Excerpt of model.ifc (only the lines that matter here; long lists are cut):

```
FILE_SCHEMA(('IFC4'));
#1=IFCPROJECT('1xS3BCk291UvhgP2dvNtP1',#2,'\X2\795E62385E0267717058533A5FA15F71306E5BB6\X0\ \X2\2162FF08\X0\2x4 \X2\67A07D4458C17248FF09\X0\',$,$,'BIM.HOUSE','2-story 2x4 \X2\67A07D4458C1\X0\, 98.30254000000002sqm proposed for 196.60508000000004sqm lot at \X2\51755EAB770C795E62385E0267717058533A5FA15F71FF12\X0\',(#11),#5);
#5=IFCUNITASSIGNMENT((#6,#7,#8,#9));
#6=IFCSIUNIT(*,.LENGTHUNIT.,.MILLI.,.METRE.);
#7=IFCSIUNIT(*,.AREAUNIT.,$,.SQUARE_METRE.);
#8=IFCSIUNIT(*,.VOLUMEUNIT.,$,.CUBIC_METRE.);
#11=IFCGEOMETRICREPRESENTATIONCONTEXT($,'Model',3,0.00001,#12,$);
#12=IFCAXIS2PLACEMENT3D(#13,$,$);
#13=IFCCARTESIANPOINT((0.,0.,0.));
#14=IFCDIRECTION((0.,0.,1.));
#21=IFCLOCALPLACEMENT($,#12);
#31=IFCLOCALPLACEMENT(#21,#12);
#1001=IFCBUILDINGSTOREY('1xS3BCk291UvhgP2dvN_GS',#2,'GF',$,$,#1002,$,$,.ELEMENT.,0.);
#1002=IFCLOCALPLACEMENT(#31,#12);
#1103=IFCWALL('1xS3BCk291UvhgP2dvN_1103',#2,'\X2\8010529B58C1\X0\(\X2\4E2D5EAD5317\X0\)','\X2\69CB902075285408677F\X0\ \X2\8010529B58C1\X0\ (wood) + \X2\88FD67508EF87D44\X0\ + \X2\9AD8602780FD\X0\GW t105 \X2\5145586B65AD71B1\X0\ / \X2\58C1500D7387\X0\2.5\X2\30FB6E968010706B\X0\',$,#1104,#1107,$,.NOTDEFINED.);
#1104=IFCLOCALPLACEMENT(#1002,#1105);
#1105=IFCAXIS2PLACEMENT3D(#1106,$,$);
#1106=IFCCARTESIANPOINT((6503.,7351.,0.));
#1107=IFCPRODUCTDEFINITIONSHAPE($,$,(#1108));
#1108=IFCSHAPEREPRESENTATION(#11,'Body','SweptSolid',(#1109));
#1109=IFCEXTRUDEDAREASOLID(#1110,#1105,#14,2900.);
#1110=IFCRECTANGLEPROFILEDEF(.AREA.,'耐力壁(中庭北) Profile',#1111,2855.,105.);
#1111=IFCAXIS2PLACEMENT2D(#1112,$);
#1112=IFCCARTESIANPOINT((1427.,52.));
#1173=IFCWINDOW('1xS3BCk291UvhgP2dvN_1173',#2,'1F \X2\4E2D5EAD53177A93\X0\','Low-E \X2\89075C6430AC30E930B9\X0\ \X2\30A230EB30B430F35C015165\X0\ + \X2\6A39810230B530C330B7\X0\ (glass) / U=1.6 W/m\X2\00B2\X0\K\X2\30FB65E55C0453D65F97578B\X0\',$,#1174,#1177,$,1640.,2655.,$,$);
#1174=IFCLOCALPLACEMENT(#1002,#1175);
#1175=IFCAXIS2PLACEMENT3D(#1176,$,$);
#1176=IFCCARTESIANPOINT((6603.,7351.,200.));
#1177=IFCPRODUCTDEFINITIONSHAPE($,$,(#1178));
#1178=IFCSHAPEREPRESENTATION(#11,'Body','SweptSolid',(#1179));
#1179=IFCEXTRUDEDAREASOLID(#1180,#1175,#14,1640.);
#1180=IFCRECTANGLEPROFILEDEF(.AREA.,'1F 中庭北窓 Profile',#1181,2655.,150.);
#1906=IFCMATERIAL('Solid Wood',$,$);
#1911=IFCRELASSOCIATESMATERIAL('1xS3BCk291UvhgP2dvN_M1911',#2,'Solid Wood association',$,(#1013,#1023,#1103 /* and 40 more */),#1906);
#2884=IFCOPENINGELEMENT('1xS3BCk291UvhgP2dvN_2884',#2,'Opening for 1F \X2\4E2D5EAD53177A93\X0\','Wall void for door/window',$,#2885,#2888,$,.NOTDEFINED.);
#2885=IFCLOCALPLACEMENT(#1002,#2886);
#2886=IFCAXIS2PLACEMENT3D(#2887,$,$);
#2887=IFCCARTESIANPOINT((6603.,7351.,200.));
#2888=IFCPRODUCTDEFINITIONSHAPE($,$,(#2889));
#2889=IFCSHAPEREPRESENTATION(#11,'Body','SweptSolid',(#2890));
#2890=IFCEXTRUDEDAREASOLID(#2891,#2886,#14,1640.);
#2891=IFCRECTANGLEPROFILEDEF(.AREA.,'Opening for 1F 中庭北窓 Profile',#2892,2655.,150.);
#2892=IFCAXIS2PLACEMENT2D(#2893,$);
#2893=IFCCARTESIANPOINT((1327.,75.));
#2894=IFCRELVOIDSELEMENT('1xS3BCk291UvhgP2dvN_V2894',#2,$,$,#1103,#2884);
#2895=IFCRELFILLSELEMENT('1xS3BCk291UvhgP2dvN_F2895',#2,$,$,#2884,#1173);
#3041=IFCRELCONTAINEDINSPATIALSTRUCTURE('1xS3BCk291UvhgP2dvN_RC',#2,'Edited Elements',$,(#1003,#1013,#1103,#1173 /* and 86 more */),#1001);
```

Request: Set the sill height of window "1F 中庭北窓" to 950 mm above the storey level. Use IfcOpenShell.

```python
import numpy as np
import ifcopenshell
import ifcopenshell.api.geometry
import ifcopenshell.geom
import ifcopenshell.util.element
import ifcopenshell.util.placement
import ifcopenshell.util.shape
import ifcopenshell.util.unit

model = ifcopenshell.open("model.ifc")
unit_scale = ifcopenshell.util.unit.calculate_unit_scale(model)

window = model.by_guid("1xS3BCk291UvhgP2dvN_1173")
opening = window.FillsVoids[0].RelatingOpeningElement
storey = ifcopenshell.util.element.get_container(window, ifc_class="IfcBuildingStorey")
level = ifcopenshell.util.placement.get_local_placement(storey.ObjectPlacement)[2, 3]

# The opening's origin need not be at the sill, so measure its lowest point.
shape = ifcopenshell.geom.create_shape(ifcopenshell.geom.settings(), opening)
bottom = ifcopenshell.util.shape.get_shape_bottom_elevation(shape, shape.geometry) / unit_scale
dz = level + 950.0 - bottom

shift = np.array([0.0, 0.0, dz])
# The window is not placed relative to its opening, so move both.
for product in (opening, window):
    matrix = ifcopenshell.util.placement.get_local_placement(product.ObjectPlacement)
    matrix[:3, 3] += shift
    ifcopenshell.api.geometry.edit_object_placement(model, product=product, matrix=matrix, is_si=False)

print(f"moved by {dz * unit_scale:+.3f} m")

model.write("model_updated.ifc")
```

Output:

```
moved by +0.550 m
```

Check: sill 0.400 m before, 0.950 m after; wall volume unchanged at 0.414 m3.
